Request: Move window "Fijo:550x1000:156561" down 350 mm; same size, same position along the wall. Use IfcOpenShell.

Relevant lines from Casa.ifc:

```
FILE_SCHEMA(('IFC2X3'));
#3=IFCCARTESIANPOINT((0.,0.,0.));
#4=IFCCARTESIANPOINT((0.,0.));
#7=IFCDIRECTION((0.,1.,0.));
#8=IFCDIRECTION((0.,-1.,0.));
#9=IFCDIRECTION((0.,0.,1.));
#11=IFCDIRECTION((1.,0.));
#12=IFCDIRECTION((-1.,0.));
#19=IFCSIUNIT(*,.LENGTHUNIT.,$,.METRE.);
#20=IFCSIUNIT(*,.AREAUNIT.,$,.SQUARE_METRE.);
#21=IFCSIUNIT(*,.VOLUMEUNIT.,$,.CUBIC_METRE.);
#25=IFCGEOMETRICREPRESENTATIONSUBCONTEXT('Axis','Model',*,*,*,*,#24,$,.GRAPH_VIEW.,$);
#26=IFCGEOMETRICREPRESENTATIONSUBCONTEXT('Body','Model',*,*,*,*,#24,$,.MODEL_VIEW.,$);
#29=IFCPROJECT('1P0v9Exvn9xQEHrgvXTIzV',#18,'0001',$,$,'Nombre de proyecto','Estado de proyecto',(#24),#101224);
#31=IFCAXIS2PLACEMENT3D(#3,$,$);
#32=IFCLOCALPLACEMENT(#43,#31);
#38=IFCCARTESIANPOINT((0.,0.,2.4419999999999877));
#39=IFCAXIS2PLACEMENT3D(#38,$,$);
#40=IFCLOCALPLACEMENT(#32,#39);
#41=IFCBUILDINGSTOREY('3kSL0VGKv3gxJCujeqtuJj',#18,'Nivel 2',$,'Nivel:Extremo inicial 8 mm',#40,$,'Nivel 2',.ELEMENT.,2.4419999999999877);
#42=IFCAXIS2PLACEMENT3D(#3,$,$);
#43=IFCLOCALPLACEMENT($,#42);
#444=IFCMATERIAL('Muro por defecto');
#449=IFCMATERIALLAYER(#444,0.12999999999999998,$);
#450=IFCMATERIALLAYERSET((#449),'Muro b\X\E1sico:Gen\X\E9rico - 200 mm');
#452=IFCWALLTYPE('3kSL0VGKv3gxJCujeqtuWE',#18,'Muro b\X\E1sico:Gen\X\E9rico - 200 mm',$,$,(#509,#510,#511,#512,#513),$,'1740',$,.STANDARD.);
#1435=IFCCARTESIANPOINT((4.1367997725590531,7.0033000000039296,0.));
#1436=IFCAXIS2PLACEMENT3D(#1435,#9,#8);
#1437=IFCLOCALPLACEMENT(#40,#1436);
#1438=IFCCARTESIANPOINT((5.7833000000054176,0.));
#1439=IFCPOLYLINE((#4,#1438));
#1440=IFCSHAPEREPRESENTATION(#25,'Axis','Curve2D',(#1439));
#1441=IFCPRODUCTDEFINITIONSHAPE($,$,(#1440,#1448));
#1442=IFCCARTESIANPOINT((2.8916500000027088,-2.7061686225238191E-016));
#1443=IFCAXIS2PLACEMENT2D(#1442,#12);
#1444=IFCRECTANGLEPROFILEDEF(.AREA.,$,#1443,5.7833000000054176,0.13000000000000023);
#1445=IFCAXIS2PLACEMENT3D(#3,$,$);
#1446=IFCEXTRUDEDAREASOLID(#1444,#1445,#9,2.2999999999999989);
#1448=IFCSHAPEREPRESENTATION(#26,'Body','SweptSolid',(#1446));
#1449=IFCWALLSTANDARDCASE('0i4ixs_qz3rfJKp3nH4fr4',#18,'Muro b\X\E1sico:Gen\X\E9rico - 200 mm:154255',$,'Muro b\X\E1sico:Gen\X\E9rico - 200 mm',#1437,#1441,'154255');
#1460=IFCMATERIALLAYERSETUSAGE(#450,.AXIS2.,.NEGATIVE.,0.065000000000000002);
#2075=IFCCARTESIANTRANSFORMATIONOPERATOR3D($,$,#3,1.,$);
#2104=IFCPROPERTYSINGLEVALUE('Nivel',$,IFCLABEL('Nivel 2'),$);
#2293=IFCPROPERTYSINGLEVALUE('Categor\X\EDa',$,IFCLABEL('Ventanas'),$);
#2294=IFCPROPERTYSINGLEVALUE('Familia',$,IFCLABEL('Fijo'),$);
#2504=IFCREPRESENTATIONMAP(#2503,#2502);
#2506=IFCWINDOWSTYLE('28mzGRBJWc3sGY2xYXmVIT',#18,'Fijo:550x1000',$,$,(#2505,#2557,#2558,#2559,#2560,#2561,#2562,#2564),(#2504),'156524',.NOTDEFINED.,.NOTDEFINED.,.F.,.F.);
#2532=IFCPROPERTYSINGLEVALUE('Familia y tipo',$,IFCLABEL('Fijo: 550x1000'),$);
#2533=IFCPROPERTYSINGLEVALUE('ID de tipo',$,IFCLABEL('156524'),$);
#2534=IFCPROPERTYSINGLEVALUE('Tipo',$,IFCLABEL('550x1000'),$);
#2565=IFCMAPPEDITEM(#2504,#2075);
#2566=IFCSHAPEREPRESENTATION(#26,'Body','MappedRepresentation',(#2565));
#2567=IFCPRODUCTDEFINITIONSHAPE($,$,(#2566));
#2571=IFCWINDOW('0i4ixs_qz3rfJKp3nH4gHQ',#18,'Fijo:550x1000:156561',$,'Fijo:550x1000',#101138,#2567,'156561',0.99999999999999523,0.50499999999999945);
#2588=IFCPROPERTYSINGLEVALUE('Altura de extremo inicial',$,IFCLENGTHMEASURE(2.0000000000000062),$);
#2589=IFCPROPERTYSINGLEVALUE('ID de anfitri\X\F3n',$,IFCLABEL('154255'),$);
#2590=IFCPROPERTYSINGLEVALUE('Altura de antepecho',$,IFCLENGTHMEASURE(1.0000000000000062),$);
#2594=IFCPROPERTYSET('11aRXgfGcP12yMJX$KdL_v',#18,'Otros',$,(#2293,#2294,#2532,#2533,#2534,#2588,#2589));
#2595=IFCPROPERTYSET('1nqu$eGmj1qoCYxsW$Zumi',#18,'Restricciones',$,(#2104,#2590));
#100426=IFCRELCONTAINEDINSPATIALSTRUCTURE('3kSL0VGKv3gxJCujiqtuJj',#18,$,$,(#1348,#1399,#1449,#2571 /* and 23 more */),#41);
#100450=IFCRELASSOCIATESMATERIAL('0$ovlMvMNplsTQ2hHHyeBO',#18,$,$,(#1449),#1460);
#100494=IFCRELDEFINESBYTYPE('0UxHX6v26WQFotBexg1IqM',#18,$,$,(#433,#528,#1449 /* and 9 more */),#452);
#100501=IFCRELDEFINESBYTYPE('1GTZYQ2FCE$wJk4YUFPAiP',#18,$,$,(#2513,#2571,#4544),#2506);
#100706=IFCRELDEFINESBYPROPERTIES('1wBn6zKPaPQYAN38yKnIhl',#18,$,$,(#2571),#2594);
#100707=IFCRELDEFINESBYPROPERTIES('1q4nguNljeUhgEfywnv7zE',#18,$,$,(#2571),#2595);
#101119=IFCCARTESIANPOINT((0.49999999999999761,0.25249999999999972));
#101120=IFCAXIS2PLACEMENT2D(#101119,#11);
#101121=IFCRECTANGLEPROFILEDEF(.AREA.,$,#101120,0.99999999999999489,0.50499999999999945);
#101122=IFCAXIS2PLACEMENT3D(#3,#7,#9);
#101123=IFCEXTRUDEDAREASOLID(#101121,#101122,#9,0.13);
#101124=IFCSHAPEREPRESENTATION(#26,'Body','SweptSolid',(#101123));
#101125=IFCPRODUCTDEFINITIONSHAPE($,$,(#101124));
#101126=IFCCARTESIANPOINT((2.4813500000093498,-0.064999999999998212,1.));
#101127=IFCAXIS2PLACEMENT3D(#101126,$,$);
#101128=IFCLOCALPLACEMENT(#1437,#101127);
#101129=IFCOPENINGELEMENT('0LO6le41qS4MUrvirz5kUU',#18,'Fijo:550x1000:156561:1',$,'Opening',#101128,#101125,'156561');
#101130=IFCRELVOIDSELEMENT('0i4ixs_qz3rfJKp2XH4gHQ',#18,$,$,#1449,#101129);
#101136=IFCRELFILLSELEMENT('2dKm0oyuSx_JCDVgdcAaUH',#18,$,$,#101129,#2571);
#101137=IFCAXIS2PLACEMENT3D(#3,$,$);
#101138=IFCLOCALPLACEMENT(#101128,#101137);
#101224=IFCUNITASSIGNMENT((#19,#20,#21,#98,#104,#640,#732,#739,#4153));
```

```python
import numpy as np
import ifcopenshell
import ifcopenshell.api.geometry
import ifcopenshell.api.pset
import ifcopenshell.util.element
import ifcopenshell.util.placement
import ifcopenshell.util.unit

model = ifcopenshell.open("Casa.ifc")
unit_scale = ifcopenshell.util.unit.calculate_unit_scale(model)

window = model.by_id(2571)
opening = window.FillsVoids[0].RelatingOpeningElement
dz = -0.35 / unit_scale

shift = np.array([0.0, 0.0, dz])
# The window is placed relative to its opening, so it follows when the opening moves.
matrix = ifcopenshell.util.placement.get_local_placement(opening.ObjectPlacement)
matrix[:3, 3] += shift
ifcopenshell.api.geometry.edit_object_placement(
    model, product=opening, matrix=matrix, is_si=False, should_transform_children=True
)

# Keep the stored heights in step.
pset = model.by_id(ifcopenshell.util.element.get_pset(window, "Otros", should_inherit=False)["id"])
ifcopenshell.api.pset.edit_pset(model, pset=pset, properties={
    "Altura de extremo inicial": model.create_entity("IfcLengthMeasure", ifcopenshell.util.element.get_pset(window, "Otros", "Altura de extremo inicial") + dz),
})
pset = model.by_id(ifcopenshell.util.element.get_pset(window, "Restricciones", should_inherit=False)["id"])
ifcopenshell.api.pset.edit_pset(model, pset=pset, properties={
    "Altura de antepecho": model.create_entity("IfcLengthMeasure", ifcopenshell.util.element.get_pset(window, "Restricciones", "Altura de antepecho") + dz),
})

print(f"moved by {dz * unit_scale:+.3f} m")

model.write("Casa_updated.ifc")
```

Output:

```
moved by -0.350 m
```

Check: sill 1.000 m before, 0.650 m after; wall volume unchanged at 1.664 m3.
